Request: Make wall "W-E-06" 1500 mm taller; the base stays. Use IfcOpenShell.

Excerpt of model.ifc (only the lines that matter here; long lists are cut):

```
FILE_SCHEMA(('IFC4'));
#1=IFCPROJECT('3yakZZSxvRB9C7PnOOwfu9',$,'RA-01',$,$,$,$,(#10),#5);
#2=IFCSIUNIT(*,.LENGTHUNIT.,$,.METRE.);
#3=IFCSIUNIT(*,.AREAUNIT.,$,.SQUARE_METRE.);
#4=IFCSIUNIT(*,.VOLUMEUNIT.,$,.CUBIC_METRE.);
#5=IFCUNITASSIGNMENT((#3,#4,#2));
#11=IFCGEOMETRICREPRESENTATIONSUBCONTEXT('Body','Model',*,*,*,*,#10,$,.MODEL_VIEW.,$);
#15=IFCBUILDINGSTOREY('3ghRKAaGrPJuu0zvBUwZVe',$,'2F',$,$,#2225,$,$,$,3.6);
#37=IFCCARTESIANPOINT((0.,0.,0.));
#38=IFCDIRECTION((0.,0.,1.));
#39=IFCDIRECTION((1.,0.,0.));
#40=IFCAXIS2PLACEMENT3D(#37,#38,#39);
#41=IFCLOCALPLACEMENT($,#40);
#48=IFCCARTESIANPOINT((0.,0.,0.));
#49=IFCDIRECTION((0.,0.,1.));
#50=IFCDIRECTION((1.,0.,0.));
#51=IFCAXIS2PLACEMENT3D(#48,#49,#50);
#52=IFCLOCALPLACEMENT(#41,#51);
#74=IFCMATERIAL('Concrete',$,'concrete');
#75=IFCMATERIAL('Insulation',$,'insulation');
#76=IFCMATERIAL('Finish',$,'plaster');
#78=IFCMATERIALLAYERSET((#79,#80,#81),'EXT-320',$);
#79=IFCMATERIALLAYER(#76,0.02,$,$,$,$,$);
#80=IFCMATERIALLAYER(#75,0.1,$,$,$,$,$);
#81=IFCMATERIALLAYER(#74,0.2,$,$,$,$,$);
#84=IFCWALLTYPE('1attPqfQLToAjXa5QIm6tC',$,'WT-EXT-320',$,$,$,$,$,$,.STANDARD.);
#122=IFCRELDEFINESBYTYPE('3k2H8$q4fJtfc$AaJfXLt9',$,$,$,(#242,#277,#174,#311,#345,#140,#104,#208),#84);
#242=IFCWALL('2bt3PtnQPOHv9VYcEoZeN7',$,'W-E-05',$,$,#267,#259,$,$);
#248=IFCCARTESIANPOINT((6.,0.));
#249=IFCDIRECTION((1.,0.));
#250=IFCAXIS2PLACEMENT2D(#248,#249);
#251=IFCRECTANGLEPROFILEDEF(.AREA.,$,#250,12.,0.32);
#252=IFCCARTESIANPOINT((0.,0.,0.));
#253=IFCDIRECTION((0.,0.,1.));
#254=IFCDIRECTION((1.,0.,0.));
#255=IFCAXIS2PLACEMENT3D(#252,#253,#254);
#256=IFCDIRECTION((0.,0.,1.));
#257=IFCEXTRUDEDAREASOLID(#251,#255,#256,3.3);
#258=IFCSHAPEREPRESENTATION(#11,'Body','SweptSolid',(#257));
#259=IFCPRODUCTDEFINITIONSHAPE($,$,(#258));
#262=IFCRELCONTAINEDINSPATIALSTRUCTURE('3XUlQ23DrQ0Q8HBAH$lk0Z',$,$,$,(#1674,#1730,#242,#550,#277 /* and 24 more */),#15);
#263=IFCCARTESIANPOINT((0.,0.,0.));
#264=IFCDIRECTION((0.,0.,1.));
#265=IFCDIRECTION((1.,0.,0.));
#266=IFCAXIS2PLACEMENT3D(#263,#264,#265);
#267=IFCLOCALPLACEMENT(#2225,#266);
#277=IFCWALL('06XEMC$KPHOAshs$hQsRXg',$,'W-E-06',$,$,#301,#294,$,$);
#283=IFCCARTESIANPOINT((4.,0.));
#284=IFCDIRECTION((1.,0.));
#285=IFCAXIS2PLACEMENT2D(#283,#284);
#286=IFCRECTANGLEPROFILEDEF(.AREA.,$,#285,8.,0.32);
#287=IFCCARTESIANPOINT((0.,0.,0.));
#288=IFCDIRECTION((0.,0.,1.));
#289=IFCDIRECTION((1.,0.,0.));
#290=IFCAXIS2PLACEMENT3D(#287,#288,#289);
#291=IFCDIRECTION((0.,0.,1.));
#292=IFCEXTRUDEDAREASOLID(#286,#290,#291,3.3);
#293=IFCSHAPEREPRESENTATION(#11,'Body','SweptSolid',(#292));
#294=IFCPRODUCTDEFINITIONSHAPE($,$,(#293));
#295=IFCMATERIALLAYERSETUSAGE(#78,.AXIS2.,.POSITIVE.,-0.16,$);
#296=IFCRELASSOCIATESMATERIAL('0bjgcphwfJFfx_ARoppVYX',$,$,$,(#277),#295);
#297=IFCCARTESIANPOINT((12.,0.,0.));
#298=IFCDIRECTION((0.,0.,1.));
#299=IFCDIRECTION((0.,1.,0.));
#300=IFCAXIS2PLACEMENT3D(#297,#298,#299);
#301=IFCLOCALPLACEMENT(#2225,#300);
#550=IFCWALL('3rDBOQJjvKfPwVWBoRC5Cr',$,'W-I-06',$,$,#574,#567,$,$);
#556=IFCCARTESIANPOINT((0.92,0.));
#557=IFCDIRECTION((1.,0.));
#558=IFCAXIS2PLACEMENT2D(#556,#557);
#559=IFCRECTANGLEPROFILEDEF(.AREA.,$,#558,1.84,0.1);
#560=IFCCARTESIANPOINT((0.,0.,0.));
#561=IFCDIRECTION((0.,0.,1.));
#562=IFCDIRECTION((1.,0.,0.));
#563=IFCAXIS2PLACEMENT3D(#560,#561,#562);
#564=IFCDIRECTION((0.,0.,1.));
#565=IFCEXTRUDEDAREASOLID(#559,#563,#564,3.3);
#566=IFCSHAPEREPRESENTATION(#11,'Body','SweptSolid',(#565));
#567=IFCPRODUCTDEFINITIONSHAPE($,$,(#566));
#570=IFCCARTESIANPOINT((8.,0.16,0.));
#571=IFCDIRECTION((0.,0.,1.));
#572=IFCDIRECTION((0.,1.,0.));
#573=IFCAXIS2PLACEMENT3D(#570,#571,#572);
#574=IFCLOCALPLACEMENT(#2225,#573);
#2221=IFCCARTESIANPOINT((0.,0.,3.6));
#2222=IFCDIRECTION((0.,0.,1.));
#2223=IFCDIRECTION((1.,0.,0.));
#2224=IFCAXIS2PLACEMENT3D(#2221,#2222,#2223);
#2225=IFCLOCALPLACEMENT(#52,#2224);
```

```python
import ifcopenshell
import ifcopenshell.geom
import ifcopenshell.util.representation
import ifcopenshell.util.shape
import ifcopenshell.util.unit

model = ifcopenshell.open("model.ifc")
unit_scale = ifcopenshell.util.unit.calculate_unit_scale(model)
settings = ifcopenshell.geom.settings()


def volume(element):
    """Net volume in cubic metres, openings subtracted."""
    shape = ifcopenshell.geom.create_shape(settings, element)
    return ifcopenshell.util.shape.get_volume(shape.geometry)


wall = model.by_guid("06XEMC$KPHOAshs$hQsRXg")
before = volume(wall)

body = ifcopenshell.util.representation.get_representation(wall, "Model", "Body")
solid = body.Items[0]
old_height = solid.Depth
solid.Depth += 1.5 / unit_scale
after = volume(wall)

print(f"height {old_height:g} -> {solid.Depth:g}, volume {before:.3f} -> {after:.3f} m3")

model.write("model_rev.ifc")
```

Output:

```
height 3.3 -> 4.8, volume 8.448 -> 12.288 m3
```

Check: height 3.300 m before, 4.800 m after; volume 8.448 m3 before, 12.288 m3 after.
